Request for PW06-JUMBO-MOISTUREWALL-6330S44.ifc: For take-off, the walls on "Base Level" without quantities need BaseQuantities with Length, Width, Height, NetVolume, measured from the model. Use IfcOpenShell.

First a look at what the model holds.

```python
import ifcopenshell
import ifcopenshell.util.element
import ifcopenshell.util.unit

model = ifcopenshell.open("PW06-JUMBO-MOISTUREWALL-6330S44.ifc")
print(model.schema)
for unit_type in ("LENGTHUNIT", "AREAUNIT", "VOLUMEUNIT"):
    print(unit_type, ifcopenshell.util.unit.calculate_unit_scale(model, unit_type))
storey = next(s for s in model.by_type("IfcBuildingStorey") if s.Name == "Base Level")
walls = [e for e in ifcopenshell.util.element.get_decomposition(storey) if e.is_a("IfcWall")]
for e in sorted(walls, key=lambda e: e.id()):
    print(e.id(), e.is_a(), e.Name, list(ifcopenshell.util.element.get_psets(e, qtos_only=True)), sep=" | ")
```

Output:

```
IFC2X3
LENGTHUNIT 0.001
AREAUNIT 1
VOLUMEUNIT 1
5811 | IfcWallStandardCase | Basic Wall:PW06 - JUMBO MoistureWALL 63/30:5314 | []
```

```python
import ifcopenshell
import ifcopenshell.api.pset
import ifcopenshell.geom
import ifcopenshell.util.element
import ifcopenshell.util.shape
import ifcopenshell.util.unit

model = ifcopenshell.open("PW06-JUMBO-MOISTUREWALL-6330S44.ifc")
unit_scale = ifcopenshell.util.unit.calculate_unit_scale(model)
volume_scale = ifcopenshell.util.unit.calculate_unit_scale(model, "VOLUMEUNIT")
settings = ifcopenshell.geom.settings()

storey = next(s for s in model.by_type("IfcBuildingStorey") if s.Name == "Base Level")
walls = [e for e in ifcopenshell.util.element.get_decomposition(storey) if e.is_a("IfcWall")]

for e in sorted(walls, key=lambda e: e.id()):
    if ifcopenshell.util.element.get_psets(e, qtos_only=True, should_inherit=False):
        continue
    # Geometry comes back in metres, in the element's own axes.
    shape = ifcopenshell.geom.create_shape(settings, e)
    values = {
        "Length": ifcopenshell.util.shape.get_x(shape.geometry) / unit_scale,
        "Width": ifcopenshell.util.shape.get_y(shape.geometry) / unit_scale,
        "Height": ifcopenshell.util.shape.get_z(shape.geometry) / unit_scale,
        "NetVolume": ifcopenshell.util.shape.get_volume(shape.geometry) / volume_scale,
    }
    qto = ifcopenshell.api.pset.add_qto(model, product=e, name="BaseQuantities")
    ifcopenshell.api.pset.edit_qto(model, qto=qto, properties=values)
    print(e.id(), {k: round(v, 3) for k, v in values.items()})

model.write("PW06-JUMBO-MOISTUREWALL-6330S44_rev.ifc")
```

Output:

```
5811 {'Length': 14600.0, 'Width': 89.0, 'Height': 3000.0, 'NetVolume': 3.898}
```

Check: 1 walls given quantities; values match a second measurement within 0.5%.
